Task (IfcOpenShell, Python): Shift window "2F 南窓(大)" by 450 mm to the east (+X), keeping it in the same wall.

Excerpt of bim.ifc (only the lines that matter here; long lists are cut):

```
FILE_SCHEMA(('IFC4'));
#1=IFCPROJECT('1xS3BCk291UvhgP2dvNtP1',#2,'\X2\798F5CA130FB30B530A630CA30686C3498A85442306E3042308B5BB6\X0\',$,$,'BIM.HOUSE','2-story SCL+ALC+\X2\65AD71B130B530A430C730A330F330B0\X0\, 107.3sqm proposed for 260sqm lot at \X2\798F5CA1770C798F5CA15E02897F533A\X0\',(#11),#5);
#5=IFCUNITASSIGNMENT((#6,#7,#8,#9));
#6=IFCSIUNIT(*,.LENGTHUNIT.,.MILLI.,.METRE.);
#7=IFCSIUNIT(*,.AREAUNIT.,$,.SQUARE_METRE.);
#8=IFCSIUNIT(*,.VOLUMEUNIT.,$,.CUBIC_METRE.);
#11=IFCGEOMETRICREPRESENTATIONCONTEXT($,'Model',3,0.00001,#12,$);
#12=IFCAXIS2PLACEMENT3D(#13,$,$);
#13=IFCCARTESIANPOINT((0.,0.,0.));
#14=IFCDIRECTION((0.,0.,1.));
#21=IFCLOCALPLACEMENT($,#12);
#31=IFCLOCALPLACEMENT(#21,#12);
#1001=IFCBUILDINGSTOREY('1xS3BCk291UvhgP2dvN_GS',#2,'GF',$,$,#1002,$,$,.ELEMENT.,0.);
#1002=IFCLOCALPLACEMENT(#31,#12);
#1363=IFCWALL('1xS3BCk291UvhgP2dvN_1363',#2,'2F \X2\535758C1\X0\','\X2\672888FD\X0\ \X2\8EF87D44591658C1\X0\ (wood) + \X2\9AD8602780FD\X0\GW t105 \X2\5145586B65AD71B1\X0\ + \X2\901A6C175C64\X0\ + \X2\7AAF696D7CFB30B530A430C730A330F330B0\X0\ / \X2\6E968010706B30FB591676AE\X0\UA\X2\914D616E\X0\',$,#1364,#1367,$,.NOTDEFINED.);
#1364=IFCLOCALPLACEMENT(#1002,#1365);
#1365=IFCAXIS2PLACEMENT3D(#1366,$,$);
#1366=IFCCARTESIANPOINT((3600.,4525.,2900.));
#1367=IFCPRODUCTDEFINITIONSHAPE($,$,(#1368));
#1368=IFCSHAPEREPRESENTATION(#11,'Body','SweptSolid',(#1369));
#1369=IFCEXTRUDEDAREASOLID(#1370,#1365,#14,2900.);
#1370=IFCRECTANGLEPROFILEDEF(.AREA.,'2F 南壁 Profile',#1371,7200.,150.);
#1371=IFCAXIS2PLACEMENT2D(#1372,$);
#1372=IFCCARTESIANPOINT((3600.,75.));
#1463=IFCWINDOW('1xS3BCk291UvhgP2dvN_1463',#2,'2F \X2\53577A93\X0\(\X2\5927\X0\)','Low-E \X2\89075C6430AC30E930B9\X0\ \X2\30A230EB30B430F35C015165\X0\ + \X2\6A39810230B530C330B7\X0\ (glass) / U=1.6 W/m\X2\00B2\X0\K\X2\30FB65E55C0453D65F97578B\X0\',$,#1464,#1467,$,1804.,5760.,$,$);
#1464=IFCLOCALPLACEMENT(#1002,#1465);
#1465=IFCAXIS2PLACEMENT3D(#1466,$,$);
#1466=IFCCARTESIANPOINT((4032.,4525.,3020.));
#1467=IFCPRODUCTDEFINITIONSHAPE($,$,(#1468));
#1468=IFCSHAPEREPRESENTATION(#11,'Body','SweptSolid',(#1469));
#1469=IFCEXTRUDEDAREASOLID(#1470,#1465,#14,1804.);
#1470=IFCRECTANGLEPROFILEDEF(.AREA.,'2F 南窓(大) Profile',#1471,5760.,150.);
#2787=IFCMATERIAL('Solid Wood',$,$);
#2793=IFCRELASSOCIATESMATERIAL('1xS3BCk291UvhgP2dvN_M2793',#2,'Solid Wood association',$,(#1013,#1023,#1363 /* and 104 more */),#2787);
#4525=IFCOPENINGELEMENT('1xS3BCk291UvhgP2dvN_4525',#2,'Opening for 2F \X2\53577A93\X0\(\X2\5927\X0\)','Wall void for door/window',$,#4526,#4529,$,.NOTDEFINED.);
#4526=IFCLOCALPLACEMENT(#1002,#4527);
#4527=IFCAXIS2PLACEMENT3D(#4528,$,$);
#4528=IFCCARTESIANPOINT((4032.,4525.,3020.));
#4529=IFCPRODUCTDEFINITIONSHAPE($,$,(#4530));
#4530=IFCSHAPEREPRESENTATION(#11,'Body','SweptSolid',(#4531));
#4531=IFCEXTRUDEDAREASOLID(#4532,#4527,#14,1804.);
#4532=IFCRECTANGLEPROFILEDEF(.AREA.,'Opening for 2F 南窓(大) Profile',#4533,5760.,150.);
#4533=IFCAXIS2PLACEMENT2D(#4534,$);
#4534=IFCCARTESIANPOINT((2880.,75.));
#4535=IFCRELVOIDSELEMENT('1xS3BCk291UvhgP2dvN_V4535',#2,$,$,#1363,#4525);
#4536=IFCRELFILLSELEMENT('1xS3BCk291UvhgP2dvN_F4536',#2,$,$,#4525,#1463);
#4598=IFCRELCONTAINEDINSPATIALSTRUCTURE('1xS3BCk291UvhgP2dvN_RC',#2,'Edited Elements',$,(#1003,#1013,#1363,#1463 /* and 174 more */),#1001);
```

```python
import ifcopenshell
import ifcopenshell.api.geometry
import ifcopenshell.util.placement

model = ifcopenshell.open("bim.ifc")

window = model.by_id(1463)
opening = window.FillsVoids[0].RelatingOpeningElement
wall = opening.VoidsElements[0].RelatingBuildingElement

wall_matrix = ifcopenshell.util.placement.get_local_placement(wall.ObjectPlacement)
shift = wall_matrix[:3, 0] * 450.0
before = ifcopenshell.util.placement.get_local_placement(window.ObjectPlacement)[:3, 3].copy()

# The window is not placed relative to its opening, so move both.
for product in (opening, window):
    matrix = ifcopenshell.util.placement.get_local_placement(product.ObjectPlacement)
    matrix[:3, 3] += shift
    ifcopenshell.api.geometry.edit_object_placement(model, product=product, matrix=matrix, is_si=False)

after = ifcopenshell.util.placement.get_local_placement(window.ObjectPlacement)[:3, 3]
print("window moved by", (after - before).round(3) + 0.0)

model.write("bim_rev.ifc")
```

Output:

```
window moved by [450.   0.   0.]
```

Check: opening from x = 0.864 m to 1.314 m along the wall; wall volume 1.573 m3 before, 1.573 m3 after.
